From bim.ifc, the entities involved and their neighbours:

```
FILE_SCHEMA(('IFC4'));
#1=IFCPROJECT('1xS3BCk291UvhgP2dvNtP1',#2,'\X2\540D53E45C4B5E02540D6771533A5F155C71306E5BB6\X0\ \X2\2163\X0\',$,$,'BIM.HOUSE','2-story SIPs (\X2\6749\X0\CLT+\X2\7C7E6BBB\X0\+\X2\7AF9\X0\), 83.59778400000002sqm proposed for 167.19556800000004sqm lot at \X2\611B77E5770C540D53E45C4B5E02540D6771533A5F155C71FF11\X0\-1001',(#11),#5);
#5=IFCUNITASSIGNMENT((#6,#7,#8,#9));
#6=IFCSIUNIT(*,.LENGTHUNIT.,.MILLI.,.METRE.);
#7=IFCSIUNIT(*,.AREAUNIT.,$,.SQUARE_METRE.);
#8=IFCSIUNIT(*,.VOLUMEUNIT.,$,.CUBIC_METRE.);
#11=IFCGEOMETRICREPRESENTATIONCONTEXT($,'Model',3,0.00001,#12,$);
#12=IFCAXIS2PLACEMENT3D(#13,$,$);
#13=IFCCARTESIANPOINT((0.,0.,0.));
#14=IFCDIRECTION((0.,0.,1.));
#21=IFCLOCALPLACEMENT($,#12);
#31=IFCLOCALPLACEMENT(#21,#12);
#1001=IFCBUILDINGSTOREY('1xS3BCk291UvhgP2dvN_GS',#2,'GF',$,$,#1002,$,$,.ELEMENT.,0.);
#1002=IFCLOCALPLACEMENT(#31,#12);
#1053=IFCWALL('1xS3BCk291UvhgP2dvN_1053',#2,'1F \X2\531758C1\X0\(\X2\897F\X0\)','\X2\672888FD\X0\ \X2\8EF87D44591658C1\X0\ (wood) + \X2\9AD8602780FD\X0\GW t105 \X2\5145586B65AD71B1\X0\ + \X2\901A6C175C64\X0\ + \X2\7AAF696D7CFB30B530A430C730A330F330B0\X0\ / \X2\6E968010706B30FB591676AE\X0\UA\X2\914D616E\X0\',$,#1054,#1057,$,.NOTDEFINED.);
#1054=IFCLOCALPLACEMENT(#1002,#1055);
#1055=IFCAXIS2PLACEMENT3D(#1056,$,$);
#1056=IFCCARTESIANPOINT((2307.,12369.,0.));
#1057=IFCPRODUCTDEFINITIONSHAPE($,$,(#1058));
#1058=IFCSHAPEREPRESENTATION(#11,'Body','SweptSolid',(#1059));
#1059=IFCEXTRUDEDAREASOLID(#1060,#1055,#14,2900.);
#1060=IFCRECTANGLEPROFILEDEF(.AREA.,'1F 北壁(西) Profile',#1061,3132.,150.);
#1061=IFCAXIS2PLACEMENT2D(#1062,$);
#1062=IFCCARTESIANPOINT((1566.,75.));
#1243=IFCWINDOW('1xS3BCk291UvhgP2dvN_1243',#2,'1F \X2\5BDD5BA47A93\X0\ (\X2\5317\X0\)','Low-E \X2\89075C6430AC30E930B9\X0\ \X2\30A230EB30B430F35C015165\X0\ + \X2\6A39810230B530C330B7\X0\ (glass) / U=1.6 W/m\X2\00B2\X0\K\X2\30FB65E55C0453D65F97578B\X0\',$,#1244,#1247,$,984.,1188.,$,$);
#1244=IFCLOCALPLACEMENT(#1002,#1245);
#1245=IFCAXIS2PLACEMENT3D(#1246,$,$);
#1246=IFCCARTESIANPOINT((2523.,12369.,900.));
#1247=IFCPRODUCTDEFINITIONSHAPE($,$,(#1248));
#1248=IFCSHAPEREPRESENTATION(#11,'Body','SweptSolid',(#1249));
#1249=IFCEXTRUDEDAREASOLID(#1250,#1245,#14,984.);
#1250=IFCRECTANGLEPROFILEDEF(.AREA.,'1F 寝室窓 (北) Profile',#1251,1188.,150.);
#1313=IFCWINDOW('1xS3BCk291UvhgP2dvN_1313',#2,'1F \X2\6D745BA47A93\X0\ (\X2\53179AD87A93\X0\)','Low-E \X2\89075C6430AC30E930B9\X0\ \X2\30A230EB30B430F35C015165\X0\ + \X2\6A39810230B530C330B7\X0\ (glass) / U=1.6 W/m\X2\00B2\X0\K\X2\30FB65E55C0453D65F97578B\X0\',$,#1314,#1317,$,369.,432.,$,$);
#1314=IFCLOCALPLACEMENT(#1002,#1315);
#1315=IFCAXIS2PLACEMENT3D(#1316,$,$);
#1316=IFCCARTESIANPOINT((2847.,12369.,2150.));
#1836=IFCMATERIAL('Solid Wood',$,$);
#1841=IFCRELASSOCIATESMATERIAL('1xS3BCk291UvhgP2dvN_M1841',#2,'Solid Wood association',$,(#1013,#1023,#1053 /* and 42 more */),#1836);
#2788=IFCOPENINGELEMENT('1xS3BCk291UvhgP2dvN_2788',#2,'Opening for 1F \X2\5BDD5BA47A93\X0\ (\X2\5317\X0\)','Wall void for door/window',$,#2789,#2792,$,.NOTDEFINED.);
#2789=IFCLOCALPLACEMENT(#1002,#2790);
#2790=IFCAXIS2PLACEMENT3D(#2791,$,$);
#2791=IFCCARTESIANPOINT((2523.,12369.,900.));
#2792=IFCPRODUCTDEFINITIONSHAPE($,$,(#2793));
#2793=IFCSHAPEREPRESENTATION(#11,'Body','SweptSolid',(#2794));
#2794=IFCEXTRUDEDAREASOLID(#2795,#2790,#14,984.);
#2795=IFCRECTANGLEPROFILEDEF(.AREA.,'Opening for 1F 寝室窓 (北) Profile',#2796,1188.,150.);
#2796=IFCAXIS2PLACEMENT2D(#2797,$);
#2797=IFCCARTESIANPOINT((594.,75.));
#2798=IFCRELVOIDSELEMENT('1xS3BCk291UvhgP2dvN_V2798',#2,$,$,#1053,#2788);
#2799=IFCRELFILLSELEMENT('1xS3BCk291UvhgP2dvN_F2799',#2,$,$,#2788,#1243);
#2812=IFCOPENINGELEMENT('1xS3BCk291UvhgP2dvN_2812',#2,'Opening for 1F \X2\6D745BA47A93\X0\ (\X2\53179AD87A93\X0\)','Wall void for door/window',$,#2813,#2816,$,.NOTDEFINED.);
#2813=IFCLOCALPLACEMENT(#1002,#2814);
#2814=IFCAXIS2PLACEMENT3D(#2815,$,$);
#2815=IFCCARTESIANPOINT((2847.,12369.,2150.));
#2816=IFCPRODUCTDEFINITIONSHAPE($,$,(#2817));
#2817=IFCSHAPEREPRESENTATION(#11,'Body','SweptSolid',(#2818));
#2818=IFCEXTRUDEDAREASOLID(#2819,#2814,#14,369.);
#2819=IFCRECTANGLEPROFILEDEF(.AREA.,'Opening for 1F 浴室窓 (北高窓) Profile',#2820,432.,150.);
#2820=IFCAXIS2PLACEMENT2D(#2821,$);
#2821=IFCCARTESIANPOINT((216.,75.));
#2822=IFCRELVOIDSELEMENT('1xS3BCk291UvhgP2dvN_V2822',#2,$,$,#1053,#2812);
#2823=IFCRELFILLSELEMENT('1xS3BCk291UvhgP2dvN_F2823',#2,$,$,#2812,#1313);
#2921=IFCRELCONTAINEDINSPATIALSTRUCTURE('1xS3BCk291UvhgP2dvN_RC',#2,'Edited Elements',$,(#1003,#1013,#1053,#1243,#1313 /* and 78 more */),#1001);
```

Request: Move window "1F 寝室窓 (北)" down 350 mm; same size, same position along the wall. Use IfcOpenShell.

```python
import numpy as np
import ifcopenshell
import ifcopenshell.api.geometry
import ifcopenshell.util.placement
import ifcopenshell.util.unit

model = ifcopenshell.open("bim.ifc")
unit_scale = ifcopenshell.util.unit.calculate_unit_scale(model)

window = model.by_guid("1xS3BCk291UvhgP2dvN_1243")
opening = window.FillsVoids[0].RelatingOpeningElement
dz = -350.0

shift = np.array([0.0, 0.0, dz])
# The window is not placed relative to its opening, so move both.
for product in (opening, window):
    matrix = ifcopenshell.util.placement.get_local_placement(product.ObjectPlacement)
    matrix[:3, 3] += shift
    ifcopenshell.api.geometry.edit_object_placement(model, product=product, matrix=matrix, is_si=False)

print(f"moved by {dz * unit_scale:+.3f} m")

model.write("bim_rev.ifc")
```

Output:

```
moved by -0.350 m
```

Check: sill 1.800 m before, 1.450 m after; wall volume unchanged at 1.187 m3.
